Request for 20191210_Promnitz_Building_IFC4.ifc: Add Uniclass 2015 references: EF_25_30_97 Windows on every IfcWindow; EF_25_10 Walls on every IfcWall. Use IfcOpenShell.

First a look at what the model holds.

```python
import ifcopenshell

model = ifcopenshell.open("20191210_Promnitz_Building_IFC4.ifc")
print(model.schema)
print("classifications:", [c.Name for c in model.by_type("IfcClassification")])
for ifc_class in ("IfcDoor", "IfcRoof", "IfcStair", "IfcWall", "IfcWindow"):
    print(ifc_class, len(model.by_type(ifc_class)))
```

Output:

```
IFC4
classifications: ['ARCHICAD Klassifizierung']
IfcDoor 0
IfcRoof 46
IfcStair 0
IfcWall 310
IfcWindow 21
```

```python
import ifcopenshell
import ifcopenshell.api.classification

model = ifcopenshell.open("20191210_Promnitz_Building_IFC4.ifc")

system = ifcopenshell.api.classification.add_classification(model, classification="Uniclass 2015")

codes = {
    "IfcWindow": ("EF_25_30_97", "Windows"),
    "IfcWall": ("EF_25_10", "Walls"),
}
for ifc_class, (code, name) in codes.items():
    products = model.by_type(ifc_class)
    ifcopenshell.api.classification.add_reference(
        model, products=products, classification=system, identification=code, name=name
    )
    print(code, len(products))

model.write("20191210_Promnitz_Building_IFC4_rev.ifc")
```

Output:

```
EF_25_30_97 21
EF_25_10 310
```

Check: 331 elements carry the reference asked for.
